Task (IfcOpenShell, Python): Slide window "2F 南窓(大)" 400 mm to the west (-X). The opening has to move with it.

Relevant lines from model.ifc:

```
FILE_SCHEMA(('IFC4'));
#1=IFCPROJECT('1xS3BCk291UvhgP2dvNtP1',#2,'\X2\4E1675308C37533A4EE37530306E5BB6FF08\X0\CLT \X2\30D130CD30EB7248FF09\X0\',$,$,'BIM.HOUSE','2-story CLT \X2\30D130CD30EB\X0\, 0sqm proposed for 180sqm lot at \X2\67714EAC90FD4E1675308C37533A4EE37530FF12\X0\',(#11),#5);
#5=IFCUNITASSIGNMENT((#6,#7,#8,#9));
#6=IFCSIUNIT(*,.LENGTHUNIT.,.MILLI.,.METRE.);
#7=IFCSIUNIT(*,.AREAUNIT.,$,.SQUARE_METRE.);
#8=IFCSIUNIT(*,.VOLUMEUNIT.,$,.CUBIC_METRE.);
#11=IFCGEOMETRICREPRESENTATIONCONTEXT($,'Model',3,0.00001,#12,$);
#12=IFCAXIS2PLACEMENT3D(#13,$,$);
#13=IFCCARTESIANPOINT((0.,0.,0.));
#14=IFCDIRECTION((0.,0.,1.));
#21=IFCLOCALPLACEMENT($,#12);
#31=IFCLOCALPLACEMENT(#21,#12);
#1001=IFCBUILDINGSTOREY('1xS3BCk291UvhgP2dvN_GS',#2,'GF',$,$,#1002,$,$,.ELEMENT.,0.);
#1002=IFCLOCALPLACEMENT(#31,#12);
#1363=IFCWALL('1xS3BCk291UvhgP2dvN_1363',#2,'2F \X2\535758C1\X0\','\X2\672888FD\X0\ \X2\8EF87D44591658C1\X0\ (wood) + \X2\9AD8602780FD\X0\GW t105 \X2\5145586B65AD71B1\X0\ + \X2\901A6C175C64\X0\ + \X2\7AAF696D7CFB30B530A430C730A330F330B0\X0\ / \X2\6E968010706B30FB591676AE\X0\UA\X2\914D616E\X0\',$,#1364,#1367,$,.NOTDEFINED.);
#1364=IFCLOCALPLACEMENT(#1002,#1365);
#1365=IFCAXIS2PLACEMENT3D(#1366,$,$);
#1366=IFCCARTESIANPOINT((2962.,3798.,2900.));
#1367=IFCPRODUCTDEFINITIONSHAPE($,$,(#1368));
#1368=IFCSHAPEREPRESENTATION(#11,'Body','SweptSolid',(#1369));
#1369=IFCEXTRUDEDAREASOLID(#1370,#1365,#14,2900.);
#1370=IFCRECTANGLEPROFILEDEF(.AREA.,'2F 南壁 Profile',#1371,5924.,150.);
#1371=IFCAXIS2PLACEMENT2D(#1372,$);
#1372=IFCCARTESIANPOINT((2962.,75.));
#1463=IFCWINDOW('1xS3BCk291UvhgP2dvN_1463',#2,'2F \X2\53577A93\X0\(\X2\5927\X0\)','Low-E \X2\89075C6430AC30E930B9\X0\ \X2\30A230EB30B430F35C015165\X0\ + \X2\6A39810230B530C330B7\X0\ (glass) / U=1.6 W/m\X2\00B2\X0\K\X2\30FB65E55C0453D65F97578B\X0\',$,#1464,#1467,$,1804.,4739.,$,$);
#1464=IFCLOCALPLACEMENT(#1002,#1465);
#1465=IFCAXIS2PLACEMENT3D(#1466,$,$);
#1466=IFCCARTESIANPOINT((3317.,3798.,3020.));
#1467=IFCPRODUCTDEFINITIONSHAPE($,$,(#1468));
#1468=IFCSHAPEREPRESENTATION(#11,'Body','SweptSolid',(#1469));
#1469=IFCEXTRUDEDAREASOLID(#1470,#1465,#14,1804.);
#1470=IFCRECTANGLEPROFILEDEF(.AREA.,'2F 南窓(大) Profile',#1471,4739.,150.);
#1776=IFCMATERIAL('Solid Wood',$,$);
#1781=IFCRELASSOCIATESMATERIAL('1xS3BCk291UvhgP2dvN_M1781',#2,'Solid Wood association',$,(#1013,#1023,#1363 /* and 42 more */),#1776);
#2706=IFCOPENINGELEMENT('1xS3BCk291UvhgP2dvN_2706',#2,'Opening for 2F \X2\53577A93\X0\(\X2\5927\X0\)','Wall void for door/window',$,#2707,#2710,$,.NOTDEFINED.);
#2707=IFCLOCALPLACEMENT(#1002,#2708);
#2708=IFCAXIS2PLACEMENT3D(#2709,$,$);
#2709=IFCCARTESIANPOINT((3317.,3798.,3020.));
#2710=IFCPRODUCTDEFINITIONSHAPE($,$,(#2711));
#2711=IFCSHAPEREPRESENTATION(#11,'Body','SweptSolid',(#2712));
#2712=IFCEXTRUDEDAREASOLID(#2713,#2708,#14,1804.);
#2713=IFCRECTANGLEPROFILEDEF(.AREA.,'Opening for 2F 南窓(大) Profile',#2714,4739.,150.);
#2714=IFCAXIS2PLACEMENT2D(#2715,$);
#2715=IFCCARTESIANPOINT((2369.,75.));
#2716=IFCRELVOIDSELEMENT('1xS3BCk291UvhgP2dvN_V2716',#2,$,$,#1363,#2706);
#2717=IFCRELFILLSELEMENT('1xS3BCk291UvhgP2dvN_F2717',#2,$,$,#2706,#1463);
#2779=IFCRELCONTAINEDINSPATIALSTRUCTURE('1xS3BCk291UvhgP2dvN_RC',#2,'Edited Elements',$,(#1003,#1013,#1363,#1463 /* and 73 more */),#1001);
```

```python
import ifcopenshell
import ifcopenshell.api.geometry
import ifcopenshell.util.placement
import ifcopenshell.util.unit

model = ifcopenshell.open("model.ifc")
unit_scale = ifcopenshell.util.unit.calculate_unit_scale(model)

window = model.by_guid("1xS3BCk291UvhgP2dvN_1463")
opening = window.FillsVoids[0].RelatingOpeningElement
wall = opening.VoidsElements[0].RelatingBuildingElement

wall_matrix = ifcopenshell.util.placement.get_local_placement(wall.ObjectPlacement)
shift = wall_matrix[:3, 0] * -0.4 / unit_scale
before = ifcopenshell.util.placement.get_local_placement(window.ObjectPlacement)[:3, 3].copy()

# The window is not placed relative to its opening, so move both.
for product in (opening, window):
    matrix = ifcopenshell.util.placement.get_local_placement(product.ObjectPlacement)
    matrix[:3, 3] += shift
    ifcopenshell.api.geometry.edit_object_placement(model, product=product, matrix=matrix, is_si=False)

after = ifcopenshell.util.placement.get_local_placement(window.ObjectPlacement)[:3, 3]
print("window moved by", (after - before).round(3) + 0.0)

model.write("model_updated.ifc")
```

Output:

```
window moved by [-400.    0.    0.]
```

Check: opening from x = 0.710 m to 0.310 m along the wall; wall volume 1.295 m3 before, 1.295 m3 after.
